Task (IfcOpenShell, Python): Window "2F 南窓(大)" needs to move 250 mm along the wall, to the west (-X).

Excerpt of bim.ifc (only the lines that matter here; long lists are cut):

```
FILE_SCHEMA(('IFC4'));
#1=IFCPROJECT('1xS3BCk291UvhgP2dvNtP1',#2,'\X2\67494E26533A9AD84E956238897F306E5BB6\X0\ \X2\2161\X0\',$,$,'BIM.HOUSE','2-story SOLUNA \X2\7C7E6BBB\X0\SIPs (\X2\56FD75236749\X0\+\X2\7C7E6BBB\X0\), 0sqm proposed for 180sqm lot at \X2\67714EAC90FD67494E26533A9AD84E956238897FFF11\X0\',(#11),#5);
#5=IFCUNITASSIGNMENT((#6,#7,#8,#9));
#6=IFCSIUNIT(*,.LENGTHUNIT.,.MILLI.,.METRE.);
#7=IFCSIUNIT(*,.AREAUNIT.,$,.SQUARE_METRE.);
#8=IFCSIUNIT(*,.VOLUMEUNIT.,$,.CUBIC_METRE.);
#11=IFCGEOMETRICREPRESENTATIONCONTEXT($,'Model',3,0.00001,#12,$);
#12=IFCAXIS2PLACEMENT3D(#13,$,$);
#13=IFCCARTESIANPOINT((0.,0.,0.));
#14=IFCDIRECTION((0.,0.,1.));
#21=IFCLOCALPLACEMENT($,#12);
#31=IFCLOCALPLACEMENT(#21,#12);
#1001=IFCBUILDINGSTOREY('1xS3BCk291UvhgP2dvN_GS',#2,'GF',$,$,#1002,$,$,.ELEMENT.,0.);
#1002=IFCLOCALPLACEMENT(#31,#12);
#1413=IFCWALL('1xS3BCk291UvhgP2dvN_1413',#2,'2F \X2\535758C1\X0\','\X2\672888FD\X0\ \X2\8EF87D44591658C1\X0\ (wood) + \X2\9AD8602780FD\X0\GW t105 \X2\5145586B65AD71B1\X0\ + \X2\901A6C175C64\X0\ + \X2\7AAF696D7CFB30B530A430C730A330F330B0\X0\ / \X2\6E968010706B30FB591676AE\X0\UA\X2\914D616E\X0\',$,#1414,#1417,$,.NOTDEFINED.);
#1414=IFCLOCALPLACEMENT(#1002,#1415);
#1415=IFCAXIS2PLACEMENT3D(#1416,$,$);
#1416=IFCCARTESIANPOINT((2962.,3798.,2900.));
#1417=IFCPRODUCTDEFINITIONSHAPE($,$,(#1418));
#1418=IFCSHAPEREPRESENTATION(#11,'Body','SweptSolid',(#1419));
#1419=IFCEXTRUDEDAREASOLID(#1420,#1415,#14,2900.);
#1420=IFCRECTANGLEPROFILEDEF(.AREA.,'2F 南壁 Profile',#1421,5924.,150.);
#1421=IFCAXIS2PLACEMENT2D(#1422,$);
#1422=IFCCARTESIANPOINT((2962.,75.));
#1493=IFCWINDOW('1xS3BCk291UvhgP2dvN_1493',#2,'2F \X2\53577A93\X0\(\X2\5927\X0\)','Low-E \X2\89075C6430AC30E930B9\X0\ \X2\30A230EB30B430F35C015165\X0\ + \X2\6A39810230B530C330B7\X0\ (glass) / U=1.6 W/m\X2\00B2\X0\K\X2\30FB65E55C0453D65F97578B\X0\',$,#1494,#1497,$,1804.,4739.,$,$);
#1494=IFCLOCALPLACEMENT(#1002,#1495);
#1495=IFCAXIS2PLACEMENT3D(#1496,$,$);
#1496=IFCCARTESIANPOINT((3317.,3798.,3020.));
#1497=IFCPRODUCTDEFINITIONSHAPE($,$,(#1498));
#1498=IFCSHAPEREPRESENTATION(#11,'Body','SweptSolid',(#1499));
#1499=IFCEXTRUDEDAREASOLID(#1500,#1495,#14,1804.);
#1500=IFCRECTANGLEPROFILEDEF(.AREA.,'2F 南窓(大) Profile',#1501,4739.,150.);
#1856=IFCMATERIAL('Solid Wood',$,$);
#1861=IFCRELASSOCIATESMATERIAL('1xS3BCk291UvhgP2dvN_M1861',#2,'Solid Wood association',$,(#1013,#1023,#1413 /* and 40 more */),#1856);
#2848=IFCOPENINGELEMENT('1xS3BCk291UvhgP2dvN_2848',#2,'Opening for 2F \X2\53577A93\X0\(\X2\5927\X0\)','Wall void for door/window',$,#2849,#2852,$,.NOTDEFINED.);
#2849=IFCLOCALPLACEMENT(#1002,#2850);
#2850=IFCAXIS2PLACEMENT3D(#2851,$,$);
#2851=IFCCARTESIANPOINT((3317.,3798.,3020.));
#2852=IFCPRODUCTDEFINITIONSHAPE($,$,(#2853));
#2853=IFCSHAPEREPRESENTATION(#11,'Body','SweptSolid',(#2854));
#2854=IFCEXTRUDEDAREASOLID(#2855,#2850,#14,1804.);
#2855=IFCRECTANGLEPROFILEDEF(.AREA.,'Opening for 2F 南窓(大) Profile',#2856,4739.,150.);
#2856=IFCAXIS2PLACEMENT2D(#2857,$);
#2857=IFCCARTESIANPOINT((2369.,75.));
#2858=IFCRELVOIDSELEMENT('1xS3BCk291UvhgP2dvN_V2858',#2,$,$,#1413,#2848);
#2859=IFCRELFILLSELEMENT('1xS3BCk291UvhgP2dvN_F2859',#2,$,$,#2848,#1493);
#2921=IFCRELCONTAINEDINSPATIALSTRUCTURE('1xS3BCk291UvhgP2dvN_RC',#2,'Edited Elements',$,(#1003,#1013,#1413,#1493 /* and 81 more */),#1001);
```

```python
import ifcopenshell
import ifcopenshell.api.geometry
import ifcopenshell.util.placement

model = ifcopenshell.open("bim.ifc")

window = model.by_guid("1xS3BCk291UvhgP2dvN_1493")
opening = window.FillsVoids[0].RelatingOpeningElement
wall = opening.VoidsElements[0].RelatingBuildingElement

wall_matrix = ifcopenshell.util.placement.get_local_placement(wall.ObjectPlacement)
shift = wall_matrix[:3, 0] * -250.0
before = ifcopenshell.util.placement.get_local_placement(window.ObjectPlacement)[:3, 3].copy()

# The window is not placed relative to its opening, so move both.
for product in (opening, window):
    matrix = ifcopenshell.util.placement.get_local_placement(product.ObjectPlacement)
    matrix[:3, 3] += shift
    ifcopenshell.api.geometry.edit_object_placement(model, product=product, matrix=matrix, is_si=False)

after = ifcopenshell.util.placement.get_local_placement(window.ObjectPlacement)[:3, 3]
print("window moved by", (after - before).round(3) + 0.0)

model.write("bim_v2.ifc")
```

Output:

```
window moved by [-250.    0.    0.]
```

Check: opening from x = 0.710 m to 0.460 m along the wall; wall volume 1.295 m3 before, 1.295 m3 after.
